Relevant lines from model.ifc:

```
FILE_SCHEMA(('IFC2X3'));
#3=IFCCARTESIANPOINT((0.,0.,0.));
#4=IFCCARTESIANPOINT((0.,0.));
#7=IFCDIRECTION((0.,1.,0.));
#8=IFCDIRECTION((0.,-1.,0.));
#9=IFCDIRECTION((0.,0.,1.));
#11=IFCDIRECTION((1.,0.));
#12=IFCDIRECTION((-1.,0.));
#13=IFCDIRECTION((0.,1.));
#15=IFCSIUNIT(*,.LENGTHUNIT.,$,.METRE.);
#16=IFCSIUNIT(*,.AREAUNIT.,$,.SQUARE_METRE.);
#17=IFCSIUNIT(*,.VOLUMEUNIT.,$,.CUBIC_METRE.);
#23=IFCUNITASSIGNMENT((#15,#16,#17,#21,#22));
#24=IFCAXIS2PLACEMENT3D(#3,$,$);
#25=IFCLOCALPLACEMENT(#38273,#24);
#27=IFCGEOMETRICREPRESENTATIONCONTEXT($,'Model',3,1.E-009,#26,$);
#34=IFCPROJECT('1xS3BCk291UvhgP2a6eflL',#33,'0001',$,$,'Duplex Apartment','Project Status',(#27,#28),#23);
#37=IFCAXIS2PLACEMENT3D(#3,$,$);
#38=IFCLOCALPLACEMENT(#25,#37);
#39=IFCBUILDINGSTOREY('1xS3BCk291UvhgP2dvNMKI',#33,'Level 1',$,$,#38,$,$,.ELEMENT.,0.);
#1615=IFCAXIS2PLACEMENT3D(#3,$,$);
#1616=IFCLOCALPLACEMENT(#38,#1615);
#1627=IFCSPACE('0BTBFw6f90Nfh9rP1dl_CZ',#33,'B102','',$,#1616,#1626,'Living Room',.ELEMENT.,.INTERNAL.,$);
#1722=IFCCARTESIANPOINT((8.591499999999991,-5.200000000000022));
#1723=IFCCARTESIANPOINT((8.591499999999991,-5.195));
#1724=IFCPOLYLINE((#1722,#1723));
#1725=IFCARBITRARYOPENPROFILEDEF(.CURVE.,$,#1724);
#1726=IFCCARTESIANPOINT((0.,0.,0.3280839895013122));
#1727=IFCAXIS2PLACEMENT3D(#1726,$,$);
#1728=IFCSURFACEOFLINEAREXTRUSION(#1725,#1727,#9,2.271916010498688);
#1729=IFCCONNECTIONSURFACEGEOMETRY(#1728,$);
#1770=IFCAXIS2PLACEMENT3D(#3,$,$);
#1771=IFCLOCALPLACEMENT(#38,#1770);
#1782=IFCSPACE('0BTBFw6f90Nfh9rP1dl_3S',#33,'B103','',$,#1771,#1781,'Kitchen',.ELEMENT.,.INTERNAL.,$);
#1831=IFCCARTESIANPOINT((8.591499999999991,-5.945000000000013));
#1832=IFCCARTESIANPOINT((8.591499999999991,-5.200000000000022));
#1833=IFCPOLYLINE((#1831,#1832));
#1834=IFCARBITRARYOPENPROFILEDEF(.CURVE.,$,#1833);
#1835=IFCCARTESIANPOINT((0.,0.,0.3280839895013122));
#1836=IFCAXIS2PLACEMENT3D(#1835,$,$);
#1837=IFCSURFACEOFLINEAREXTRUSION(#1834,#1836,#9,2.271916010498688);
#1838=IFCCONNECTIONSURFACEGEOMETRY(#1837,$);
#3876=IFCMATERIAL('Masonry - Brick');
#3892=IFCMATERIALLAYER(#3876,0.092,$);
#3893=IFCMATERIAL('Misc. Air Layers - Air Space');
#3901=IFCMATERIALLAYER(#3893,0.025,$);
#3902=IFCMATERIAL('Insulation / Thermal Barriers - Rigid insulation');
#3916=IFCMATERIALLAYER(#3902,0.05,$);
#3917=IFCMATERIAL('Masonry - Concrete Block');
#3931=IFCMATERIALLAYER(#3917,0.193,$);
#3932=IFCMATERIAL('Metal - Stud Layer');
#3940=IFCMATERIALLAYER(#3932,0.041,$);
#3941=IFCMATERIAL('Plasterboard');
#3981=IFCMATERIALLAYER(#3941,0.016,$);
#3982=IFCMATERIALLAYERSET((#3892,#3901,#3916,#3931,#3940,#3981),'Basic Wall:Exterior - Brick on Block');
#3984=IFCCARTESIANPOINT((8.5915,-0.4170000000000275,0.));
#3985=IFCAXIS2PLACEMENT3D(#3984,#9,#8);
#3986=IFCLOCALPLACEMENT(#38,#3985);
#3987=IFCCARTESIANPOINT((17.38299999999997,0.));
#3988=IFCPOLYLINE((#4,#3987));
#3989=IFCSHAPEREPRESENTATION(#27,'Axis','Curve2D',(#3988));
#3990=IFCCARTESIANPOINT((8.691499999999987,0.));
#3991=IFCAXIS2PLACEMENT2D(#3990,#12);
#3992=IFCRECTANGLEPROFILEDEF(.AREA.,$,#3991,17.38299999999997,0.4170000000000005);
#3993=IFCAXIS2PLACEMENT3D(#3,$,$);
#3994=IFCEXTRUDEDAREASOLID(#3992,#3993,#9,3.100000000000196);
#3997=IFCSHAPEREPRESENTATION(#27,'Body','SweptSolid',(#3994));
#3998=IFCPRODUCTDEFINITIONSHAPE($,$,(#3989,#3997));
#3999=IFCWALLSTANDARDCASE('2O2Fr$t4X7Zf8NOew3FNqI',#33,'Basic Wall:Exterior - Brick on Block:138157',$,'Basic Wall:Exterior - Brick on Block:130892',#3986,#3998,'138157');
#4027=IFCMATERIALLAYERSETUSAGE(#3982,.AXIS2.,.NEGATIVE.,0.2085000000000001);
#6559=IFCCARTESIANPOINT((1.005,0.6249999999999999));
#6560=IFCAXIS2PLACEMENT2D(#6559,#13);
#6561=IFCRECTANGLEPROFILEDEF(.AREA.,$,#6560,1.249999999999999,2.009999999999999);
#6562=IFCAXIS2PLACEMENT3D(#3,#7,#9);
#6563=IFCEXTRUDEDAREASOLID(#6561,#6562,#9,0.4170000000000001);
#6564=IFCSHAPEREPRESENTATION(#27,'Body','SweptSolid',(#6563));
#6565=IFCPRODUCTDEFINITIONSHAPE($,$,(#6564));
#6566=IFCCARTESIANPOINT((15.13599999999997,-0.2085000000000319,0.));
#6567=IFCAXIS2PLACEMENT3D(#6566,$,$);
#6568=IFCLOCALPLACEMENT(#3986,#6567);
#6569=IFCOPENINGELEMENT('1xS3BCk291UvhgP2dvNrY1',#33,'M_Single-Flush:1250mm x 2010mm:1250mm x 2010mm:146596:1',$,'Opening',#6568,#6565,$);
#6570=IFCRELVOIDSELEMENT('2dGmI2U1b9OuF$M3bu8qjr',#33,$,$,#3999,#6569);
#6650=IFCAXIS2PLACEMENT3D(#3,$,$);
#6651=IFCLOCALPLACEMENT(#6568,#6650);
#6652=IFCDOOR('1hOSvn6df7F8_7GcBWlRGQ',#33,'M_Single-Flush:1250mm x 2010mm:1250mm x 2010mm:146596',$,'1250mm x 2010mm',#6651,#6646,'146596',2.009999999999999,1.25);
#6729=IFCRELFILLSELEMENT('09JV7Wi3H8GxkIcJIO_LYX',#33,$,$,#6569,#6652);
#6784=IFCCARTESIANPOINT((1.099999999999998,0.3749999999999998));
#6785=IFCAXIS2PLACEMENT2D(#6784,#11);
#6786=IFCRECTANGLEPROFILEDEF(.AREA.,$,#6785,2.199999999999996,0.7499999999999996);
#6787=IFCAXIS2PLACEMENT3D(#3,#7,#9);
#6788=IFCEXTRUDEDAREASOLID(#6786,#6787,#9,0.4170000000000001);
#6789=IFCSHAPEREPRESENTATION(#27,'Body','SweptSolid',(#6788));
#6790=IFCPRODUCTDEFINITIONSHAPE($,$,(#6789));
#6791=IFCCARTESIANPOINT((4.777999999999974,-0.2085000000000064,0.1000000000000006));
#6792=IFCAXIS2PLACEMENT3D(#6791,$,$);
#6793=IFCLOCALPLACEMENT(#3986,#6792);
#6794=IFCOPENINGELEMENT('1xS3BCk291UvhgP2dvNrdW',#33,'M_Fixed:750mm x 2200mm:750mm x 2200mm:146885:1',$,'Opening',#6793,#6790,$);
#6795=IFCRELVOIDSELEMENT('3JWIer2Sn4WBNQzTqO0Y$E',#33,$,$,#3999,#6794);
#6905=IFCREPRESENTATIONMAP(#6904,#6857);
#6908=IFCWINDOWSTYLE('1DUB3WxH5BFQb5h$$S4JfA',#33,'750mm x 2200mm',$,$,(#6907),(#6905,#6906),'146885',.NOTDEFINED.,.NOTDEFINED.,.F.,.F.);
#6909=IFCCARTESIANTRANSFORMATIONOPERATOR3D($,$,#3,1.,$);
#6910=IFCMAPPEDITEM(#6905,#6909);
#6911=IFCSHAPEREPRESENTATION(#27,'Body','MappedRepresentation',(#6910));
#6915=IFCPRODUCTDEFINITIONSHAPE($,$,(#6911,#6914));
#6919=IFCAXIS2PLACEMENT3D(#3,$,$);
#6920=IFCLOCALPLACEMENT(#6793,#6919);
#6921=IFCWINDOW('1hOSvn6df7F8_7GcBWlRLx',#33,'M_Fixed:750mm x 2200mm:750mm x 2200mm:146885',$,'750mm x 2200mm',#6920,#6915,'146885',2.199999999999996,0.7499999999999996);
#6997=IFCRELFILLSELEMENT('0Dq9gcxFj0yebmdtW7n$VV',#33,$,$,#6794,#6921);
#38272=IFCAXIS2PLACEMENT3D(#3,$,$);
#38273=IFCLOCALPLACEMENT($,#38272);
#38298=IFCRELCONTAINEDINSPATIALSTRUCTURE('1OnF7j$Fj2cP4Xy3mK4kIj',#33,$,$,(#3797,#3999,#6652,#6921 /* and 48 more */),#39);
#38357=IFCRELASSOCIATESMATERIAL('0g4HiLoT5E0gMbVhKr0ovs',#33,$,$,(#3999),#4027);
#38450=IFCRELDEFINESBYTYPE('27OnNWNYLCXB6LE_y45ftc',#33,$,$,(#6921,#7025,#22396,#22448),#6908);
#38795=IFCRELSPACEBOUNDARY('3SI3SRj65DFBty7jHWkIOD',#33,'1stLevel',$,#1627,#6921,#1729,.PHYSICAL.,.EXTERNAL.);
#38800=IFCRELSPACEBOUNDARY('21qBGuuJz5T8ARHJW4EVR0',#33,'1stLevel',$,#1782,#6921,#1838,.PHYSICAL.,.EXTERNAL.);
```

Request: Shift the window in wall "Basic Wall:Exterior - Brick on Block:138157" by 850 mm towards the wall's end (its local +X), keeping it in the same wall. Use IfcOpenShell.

```python
import numpy as np
import ifcopenshell
import ifcopenshell.api.geometry
import ifcopenshell.util.placement

model = ifcopenshell.open("model.ifc")

window = model.by_guid("1hOSvn6df7F8_7GcBWlRLx")
opening = window.FillsVoids[0].RelatingOpeningElement
wall = opening.VoidsElements[0].RelatingBuildingElement

wall_matrix = ifcopenshell.util.placement.get_local_placement(wall.ObjectPlacement)
shift = wall_matrix[:3, 0] * 0.85
before = ifcopenshell.util.placement.get_local_placement(window.ObjectPlacement)[:3, 3].copy()

# The window is placed relative to its opening, so it follows when the opening moves.
matrix = ifcopenshell.util.placement.get_local_placement(opening.ObjectPlacement)
matrix[:3, 3] += shift
ifcopenshell.api.geometry.edit_object_placement(
    model, product=opening, matrix=matrix, is_si=False, should_transform_children=True
)

# Space boundary surfaces are stored in each space's coordinates; move them too.
for rel in window.ProvidesBoundaries:
    if not rel.ConnectionGeometry:
        continue
    surface = rel.ConnectionGeometry.SurfaceOnRelatingElement
    space_matrix = ifcopenshell.util.placement.get_local_placement(rel.RelatingSpace.ObjectPlacement)
    point = np.array(surface.Position.Location.Coordinates) + space_matrix[:3, :3].T @ shift
    surface.Position = model.createIfcAxis2Placement3D(
        model.createIfcCartesianPoint(point.tolist()), surface.Position.Axis, surface.Position.RefDirection
    )

after = ifcopenshell.util.placement.get_local_placement(window.ObjectPlacement)[:3, 3]
print("window moved by", (after - before).round(3) + 0.0)

model.write("model-out.ifc")
```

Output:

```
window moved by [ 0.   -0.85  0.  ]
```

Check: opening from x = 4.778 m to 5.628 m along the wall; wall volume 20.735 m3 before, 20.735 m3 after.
